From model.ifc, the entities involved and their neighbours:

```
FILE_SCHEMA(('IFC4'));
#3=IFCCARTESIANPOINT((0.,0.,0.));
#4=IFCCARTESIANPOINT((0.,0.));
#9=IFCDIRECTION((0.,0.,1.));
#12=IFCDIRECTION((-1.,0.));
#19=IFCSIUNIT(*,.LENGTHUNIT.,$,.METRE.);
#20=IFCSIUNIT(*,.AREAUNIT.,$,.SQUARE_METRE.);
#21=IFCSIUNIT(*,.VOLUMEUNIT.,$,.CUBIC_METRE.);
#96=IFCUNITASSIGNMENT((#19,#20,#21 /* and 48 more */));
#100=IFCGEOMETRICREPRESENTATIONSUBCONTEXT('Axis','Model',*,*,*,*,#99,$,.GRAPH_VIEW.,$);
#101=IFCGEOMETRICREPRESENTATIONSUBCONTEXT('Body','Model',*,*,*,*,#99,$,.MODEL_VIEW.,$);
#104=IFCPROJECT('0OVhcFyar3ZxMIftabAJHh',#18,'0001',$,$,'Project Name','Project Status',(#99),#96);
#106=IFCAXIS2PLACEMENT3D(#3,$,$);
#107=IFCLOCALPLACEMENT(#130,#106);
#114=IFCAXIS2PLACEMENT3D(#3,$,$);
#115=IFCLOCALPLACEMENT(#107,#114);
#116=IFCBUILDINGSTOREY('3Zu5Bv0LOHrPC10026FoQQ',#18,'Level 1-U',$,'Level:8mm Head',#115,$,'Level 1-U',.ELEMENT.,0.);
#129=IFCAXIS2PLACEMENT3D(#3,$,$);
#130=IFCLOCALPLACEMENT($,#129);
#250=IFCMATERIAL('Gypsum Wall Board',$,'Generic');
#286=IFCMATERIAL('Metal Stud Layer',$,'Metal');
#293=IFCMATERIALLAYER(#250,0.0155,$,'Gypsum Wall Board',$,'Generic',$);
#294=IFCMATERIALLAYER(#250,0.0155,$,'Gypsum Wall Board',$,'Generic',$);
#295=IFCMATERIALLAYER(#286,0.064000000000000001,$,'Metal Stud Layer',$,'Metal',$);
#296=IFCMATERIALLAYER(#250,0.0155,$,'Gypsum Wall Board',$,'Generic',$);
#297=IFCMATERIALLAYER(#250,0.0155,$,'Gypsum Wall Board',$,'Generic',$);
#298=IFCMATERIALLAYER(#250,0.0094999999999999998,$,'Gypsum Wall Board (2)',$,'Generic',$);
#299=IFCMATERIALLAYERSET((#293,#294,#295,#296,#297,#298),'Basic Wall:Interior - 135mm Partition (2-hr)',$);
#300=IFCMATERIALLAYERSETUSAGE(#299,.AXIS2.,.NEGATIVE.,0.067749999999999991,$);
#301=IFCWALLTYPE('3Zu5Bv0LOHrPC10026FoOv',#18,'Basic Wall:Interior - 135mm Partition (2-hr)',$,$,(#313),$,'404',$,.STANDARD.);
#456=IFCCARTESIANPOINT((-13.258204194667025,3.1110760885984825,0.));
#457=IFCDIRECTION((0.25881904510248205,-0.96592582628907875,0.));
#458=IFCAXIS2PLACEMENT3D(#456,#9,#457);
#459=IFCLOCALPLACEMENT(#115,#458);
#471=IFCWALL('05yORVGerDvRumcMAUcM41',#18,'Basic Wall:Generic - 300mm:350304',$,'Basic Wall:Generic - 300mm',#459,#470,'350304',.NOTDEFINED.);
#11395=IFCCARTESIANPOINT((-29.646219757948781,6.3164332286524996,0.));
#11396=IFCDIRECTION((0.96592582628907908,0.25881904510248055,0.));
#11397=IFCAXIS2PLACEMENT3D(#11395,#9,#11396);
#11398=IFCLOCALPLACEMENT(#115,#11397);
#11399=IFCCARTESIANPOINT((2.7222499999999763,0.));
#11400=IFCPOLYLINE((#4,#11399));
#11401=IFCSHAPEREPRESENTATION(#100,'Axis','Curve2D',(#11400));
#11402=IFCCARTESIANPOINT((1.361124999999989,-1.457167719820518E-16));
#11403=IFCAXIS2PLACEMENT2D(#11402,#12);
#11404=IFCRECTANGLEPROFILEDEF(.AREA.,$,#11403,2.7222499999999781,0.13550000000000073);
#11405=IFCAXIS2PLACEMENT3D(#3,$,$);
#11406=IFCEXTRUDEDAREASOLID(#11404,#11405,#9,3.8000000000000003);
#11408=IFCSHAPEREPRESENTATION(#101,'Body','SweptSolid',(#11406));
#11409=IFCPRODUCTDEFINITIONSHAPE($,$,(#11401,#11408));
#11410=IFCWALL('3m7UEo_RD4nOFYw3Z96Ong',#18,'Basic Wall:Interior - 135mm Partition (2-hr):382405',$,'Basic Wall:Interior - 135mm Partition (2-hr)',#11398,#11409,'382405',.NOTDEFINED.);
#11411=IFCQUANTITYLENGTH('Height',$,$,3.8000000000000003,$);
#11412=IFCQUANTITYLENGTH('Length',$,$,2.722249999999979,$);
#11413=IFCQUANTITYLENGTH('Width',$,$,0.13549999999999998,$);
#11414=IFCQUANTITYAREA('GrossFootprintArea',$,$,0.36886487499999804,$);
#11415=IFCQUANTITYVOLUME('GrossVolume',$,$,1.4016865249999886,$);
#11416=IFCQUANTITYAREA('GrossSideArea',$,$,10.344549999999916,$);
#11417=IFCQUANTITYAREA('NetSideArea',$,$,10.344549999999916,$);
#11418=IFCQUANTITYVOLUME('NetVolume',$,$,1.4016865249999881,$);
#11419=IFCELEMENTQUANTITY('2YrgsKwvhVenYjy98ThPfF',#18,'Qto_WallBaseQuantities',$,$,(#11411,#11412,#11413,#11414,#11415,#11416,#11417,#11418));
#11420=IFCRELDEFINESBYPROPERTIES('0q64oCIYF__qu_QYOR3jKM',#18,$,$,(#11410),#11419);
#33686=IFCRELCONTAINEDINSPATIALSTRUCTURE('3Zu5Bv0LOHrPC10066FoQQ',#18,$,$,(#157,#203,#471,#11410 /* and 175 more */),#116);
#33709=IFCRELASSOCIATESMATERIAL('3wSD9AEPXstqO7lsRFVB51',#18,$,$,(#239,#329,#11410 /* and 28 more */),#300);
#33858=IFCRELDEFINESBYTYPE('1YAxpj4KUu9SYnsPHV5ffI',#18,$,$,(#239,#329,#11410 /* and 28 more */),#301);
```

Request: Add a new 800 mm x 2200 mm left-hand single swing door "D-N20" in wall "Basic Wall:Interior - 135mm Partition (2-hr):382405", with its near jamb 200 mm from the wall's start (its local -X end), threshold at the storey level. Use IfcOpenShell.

```python
import numpy as np
import ifcopenshell
import ifcopenshell.api.feature
import ifcopenshell.api.geometry
import ifcopenshell.api.pset
import ifcopenshell.api.root
import ifcopenshell.api.spatial
import ifcopenshell.geom
import ifcopenshell.util.element
import ifcopenshell.util.placement
import ifcopenshell.util.representation
import ifcopenshell.util.shape
import ifcopenshell.util.unit

model = ifcopenshell.open("model.ifc")
unit_scale = ifcopenshell.util.unit.calculate_unit_scale(model)
area_scale = ifcopenshell.util.unit.calculate_unit_scale(model, "AREAUNIT")
volume_scale = ifcopenshell.util.unit.calculate_unit_scale(model, "VOLUMEUNIT")
settings = ifcopenshell.geom.settings()


def volume(element):
    """Net volume in cubic metres, openings subtracted."""
    shape = ifcopenshell.geom.create_shape(settings, element)
    return ifcopenshell.util.shape.get_volume(shape.geometry)


wall = model.by_id(11410)
storey = ifcopenshell.util.element.get_container(wall, ifc_class="IfcBuildingStorey")
context = ifcopenshell.util.representation.get_context(model, "Model", "Body", "MODEL_VIEW")
before = volume(wall)

width, height, from_end, sill = 0.8, 2.2, 0.2, 0.0  # metres

# The wall runs along its own X axis, and the end named is its -X end.
wall_shape = ifcopenshell.geom.create_shape(settings, wall)
x, y, z = ifcopenshell.util.shape.get_vertices(wall_shape.geometry).T
start = x.min() + from_end
face, thickness = float(y.min()), float(y.max() - y.min())
wall_matrix = ifcopenshell.util.placement.get_local_placement(wall.ObjectPlacement)
level = ifcopenshell.util.placement.get_local_placement(storey.ObjectPlacement)[2, 3]


def in_wall(x, y):
    """Placement at x, y metres in the wall's axes, at sill height."""
    matrix = wall_matrix.copy()
    matrix[:, 3] = wall_matrix @ np.array([x / unit_scale, y / unit_scale, 0.0, 1.0])
    matrix[2, 3] = level + sill / unit_scale
    return matrix


# Opening: a box that overshoots both wall faces by 50 mm.
opening = ifcopenshell.api.root.create_entity(model, ifc_class="IfcOpeningElement", predefined_type="OPENING")
box = ifcopenshell.api.geometry.add_wall_representation(
    model, context=context, length=width, height=height, thickness=thickness + 0.1
)
ifcopenshell.api.geometry.assign_representation(model, product=opening, representation=box)
ifcopenshell.api.geometry.edit_object_placement(model, product=opening, matrix=in_wall(start, face - 0.05), is_si=False)
ifcopenshell.api.feature.add_feature(model, feature=opening, element=wall)

door = ifcopenshell.api.root.create_entity(model, ifc_class="IfcDoor", name="D-N20", predefined_type="DOOR")
door.OverallWidth, door.OverallHeight = width / unit_scale, height / unit_scale
door.OperationType = "SINGLE_SWING_LEFT"
body = ifcopenshell.api.geometry.add_door_representation(
    model,
    context=context,
    overall_width=door.OverallWidth,
    overall_height=door.OverallHeight,
    operation_type="SINGLE_SWING_LEFT",
    lining_properties={"LiningDepth": thickness / unit_scale, "ThresholdDepth": thickness / unit_scale},
)
ifcopenshell.api.geometry.assign_representation(model, product=door, representation=body)
ifcopenshell.api.spatial.assign_container(model, products=[door], relating_structure=storey)
ifcopenshell.api.feature.add_filling(model, opening=opening, element=door)

# The lining spans the wall, so the door starts at the wall face.
ifcopenshell.api.geometry.edit_object_placement(model, product=door, matrix=in_wall(start, face), is_si=False)

after = volume(wall)

# Update the wall's stored quantities.
qto = model.by_id(ifcopenshell.util.element.get_pset(wall, "Qto_WallBaseQuantities", should_inherit=False)["id"])
ifcopenshell.api.pset.edit_qto(model, qto=qto, properties={
    "NetSideArea": after / thickness / area_scale,
    "NetVolume": after / volume_scale,
})

print(f"wall volume {before:.3f} -> {after:.3f} m3")

model.write("model_edited.ifc")
```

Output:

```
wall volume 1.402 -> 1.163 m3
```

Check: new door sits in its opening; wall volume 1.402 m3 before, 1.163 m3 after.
